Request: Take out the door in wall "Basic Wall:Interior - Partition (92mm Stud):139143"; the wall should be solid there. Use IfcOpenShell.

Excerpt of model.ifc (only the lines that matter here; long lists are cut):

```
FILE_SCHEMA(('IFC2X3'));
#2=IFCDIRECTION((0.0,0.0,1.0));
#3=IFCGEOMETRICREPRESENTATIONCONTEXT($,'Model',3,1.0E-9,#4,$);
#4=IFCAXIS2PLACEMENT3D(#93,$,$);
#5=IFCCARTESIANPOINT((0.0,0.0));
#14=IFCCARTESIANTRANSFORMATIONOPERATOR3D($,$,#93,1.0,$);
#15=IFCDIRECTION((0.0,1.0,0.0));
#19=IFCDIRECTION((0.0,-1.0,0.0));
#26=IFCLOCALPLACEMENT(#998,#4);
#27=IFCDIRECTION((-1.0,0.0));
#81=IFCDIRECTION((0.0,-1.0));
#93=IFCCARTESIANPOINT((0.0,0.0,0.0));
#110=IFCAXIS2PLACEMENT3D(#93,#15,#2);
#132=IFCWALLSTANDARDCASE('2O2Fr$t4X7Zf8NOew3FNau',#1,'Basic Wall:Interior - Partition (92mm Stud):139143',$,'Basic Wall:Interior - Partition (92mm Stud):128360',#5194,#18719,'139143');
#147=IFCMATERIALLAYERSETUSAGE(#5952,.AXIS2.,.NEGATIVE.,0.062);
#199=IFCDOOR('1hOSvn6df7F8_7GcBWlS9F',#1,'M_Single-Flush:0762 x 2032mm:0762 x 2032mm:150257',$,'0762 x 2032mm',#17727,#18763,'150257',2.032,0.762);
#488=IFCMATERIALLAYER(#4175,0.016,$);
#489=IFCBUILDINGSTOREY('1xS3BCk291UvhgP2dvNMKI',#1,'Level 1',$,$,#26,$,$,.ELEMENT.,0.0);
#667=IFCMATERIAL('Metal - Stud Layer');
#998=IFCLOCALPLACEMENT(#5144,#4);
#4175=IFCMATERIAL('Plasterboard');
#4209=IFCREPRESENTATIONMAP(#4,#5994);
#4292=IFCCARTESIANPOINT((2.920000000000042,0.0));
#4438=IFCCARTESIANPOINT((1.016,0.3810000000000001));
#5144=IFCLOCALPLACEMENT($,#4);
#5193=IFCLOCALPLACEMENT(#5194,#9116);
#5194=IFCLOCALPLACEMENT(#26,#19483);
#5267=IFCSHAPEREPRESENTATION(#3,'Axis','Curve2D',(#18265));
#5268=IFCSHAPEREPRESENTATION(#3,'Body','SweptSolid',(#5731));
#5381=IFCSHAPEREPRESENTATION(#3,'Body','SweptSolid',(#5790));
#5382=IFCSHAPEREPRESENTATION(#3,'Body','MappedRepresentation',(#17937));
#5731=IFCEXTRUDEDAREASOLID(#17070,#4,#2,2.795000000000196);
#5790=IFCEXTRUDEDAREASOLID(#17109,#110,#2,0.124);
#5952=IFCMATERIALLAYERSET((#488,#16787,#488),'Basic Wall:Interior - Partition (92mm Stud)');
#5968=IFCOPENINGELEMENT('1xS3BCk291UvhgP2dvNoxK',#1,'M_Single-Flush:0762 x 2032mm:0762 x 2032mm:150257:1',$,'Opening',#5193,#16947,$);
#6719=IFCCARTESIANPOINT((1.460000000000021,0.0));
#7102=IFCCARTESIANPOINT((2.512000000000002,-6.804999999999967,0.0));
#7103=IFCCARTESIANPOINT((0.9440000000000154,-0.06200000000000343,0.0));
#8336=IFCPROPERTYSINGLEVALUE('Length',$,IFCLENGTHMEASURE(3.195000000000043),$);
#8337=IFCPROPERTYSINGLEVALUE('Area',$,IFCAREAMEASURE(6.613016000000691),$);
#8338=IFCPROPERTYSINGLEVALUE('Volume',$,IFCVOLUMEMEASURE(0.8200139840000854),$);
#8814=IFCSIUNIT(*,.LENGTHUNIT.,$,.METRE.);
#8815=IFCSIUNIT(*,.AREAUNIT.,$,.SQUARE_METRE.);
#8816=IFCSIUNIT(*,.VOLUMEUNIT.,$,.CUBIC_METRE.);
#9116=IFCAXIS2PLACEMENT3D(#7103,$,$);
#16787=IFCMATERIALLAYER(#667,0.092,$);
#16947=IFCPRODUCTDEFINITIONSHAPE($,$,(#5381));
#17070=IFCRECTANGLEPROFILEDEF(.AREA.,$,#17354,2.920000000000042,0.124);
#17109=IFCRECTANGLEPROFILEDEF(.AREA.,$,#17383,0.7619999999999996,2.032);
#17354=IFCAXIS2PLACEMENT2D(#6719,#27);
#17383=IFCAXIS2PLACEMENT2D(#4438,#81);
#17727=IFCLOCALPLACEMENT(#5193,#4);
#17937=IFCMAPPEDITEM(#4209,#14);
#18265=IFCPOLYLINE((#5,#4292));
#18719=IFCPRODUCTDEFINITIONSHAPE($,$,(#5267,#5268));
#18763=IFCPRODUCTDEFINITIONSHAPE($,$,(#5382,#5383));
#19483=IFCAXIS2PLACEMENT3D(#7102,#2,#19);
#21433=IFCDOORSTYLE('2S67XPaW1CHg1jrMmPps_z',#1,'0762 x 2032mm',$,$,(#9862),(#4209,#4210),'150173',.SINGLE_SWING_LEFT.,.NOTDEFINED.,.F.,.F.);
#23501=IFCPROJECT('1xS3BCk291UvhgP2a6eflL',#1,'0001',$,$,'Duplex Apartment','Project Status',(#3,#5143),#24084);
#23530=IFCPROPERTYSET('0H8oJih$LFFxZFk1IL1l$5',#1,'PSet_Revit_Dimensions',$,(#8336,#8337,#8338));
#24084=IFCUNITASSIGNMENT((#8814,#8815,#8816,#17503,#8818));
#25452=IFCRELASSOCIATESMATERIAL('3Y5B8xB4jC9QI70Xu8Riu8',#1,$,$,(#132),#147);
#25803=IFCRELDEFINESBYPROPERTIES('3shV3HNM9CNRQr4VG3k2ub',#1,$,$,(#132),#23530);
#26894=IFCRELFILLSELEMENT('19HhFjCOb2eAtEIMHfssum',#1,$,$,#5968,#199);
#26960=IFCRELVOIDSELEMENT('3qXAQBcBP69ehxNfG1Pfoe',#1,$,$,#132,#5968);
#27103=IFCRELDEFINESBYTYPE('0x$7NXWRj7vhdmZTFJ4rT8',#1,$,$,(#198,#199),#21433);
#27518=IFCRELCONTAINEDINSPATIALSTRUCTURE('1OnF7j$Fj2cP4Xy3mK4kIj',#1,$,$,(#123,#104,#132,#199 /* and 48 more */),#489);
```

```python
import ifcopenshell
import ifcopenshell.api.feature
import ifcopenshell.api.pset
import ifcopenshell.api.root
import ifcopenshell.geom
import ifcopenshell.util.element
import ifcopenshell.util.shape
import ifcopenshell.util.unit

model = ifcopenshell.open("model.ifc")
area_scale = ifcopenshell.util.unit.calculate_unit_scale(model, "AREAUNIT")
volume_scale = ifcopenshell.util.unit.calculate_unit_scale(model, "VOLUMEUNIT")
settings = ifcopenshell.geom.settings()


def volume(element):
    """Net volume in cubic metres, openings subtracted."""
    shape = ifcopenshell.geom.create_shape(settings, element)
    return ifcopenshell.util.shape.get_volume(shape.geometry)


door = model.by_guid("1hOSvn6df7F8_7GcBWlS9F")
opening = door.FillsVoids[0].RelatingOpeningElement
wall = opening.VoidsElements[0].RelatingBuildingElement
before = volume(wall)

ifcopenshell.api.root.remove_product(model, product=door)
ifcopenshell.api.feature.remove_feature(model, feature=opening)

after = volume(wall)
thickness = 0.124  # wall thickness in metres

# Update the wall's stored quantities.
pset = model.by_id(ifcopenshell.util.element.get_pset(wall, "PSet_Revit_Dimensions", should_inherit=False)["id"])
ifcopenshell.api.pset.edit_pset(model, pset=pset, properties={
    "Area": model.create_entity("IfcAreaMeasure", after / thickness / area_scale),
    "Volume": model.create_entity("IfcVolumeMeasure", after / volume_scale),
})

print(f"wall volume {before:.3f} -> {after:.3f} m3")

model.write("model_updated.ifc")
```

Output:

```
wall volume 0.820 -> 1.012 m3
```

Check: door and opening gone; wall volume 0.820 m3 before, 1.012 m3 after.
